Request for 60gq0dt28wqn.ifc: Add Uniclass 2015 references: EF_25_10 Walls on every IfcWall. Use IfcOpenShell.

First a look at what the model holds.

```python
import ifcopenshell

model = ifcopenshell.open("60gq0dt28wqn.ifc")
print(model.schema)
print("classifications:", [c.Name for c in model.by_type("IfcClassification")])
for ifc_class in ("IfcDoor", "IfcRoof", "IfcStair", "IfcWall", "IfcWindow"):
    print(ifc_class, len(model.by_type(ifc_class)))
```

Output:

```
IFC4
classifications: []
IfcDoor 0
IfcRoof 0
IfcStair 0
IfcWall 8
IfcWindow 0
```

```python
import ifcopenshell
import ifcopenshell.api.classification

model = ifcopenshell.open("60gq0dt28wqn.ifc")

system = ifcopenshell.api.classification.add_classification(model, classification="Uniclass 2015")

codes = {
    "IfcWall": ("EF_25_10", "Walls"),
}
for ifc_class, (code, name) in codes.items():
    products = model.by_type(ifc_class)
    ifcopenshell.api.classification.add_reference(
        model, products=products, classification=system, identification=code, name=name
    )
    print(code, len(products))

model.write("60gq0dt28wqn-out.ifc")
```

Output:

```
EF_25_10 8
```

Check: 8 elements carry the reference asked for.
